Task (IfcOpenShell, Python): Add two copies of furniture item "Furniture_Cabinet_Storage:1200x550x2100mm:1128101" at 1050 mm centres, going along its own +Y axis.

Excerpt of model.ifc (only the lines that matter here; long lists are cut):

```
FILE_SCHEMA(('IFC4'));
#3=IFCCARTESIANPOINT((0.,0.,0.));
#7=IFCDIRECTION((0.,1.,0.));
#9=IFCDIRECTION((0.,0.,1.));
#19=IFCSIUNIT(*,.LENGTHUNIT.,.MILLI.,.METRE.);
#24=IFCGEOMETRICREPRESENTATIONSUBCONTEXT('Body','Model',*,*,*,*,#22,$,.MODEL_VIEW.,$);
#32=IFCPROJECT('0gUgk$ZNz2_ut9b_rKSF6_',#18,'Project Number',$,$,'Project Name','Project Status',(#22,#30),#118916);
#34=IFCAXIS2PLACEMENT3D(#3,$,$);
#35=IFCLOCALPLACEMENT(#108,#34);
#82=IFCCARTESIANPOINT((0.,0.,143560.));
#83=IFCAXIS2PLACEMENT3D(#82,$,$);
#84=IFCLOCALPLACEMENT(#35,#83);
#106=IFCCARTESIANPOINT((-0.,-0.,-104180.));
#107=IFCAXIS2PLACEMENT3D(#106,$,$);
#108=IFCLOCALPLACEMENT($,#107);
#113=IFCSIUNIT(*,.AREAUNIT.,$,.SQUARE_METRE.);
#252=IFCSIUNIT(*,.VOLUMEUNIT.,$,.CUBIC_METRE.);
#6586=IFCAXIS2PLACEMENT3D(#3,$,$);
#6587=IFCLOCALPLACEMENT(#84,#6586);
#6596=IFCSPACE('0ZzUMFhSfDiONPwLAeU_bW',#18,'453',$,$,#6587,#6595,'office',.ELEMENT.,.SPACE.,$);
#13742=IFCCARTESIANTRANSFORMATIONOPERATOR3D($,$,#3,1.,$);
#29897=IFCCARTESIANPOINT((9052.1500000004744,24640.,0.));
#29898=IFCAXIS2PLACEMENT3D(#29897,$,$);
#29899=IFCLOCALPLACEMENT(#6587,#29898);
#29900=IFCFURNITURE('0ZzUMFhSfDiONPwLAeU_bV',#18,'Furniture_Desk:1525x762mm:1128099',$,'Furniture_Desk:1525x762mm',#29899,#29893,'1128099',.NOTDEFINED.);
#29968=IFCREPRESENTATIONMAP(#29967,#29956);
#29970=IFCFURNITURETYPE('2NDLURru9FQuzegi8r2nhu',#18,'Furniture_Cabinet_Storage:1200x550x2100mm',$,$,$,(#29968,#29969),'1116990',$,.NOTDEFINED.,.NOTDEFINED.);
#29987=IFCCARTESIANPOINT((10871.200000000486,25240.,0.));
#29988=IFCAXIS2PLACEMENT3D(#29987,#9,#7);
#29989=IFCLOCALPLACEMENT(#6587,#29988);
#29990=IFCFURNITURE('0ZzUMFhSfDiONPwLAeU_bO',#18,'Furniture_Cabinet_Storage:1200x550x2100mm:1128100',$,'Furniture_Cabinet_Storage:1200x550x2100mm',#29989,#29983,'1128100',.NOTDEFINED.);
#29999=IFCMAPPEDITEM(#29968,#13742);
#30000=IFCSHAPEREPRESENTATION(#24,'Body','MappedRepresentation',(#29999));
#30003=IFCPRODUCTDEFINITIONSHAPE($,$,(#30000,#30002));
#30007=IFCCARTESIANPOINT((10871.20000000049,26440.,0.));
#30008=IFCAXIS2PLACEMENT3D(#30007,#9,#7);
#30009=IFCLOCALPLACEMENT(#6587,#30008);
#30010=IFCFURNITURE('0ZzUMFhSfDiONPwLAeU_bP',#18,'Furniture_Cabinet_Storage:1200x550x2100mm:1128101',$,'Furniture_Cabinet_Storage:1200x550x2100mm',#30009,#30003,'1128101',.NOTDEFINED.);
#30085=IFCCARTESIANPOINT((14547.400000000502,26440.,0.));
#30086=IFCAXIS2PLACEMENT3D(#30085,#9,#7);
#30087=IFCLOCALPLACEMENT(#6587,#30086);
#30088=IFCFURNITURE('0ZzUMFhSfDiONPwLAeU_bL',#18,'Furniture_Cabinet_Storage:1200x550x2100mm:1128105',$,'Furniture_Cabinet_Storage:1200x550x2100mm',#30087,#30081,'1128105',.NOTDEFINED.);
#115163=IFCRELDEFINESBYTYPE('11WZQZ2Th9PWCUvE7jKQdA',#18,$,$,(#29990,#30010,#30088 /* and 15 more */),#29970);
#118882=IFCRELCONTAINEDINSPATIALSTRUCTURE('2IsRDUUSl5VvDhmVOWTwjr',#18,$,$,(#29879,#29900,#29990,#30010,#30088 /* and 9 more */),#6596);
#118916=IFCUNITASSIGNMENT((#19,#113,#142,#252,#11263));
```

```python
import ifcopenshell
import ifcopenshell.api.geometry
import ifcopenshell.api.root
import ifcopenshell.util.element
import ifcopenshell.util.placement

model = ifcopenshell.open("model.ifc")


def reuse_history(source, copy):
    """copy_class also copies each property set's owner history, people and application; keep the originals."""
    for rel in copy.IsDefinedBy:
        if rel.is_a("IfcRelDefinesByProperties") and (history := rel.RelatingPropertyDefinition.OwnerHistory):
            rel.RelatingPropertyDefinition.OwnerHistory = source.OwnerHistory
            ifcopenshell.util.element.remove_deep2(model, history)


source = model.by_guid("0ZzUMFhSfDiONPwLAeU_bP")
base = ifcopenshell.util.placement.get_local_placement(source.ObjectPlacement)
step = base[:3, 1] * 1050.0

for i in range(1, 3):
    copy = ifcopenshell.api.root.copy_class(model, product=source)
    copy.Representation = ifcopenshell.util.element.copy_deep(
        model, source.Representation, exclude=["IfcGeometricRepresentationContext", "IfcRepresentationMap"]
    )
    copy.Name = "Furniture_Cabinet_Storage:1200x550x2100mm"
    copy.Tag = None
    reuse_history(source, copy)
    matrix = base.copy()
    matrix[:3, 3] += i * step
    print("added at", matrix[:3, 3].round(3) + 0.0)
    ifcopenshell.api.geometry.edit_object_placement(model, product=copy, matrix=matrix, is_si=False)

model.write("model_updated.ifc")
```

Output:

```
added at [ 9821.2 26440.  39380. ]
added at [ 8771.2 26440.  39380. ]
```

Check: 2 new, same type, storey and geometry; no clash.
